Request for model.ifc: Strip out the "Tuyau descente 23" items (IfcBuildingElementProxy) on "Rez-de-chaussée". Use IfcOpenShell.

First a look at what the model holds.

```python
import ifcopenshell
import ifcopenshell.util.element

model = ifcopenshell.open("model.ifc")
print(model.schema)
storey = next(s for s in model.by_type("IfcBuildingStorey") if s.Name == "Rez-de-chaussée")
proxies = [e for e in ifcopenshell.util.element.get_decomposition(storey) if e.is_a("IfcBuildingElementProxy")]
seen = {}
for e in proxies:
    element_type = ifcopenshell.util.element.get_type(e)
    name = element_type.Name if element_type not in (None, e) else None
    seen[name] = seen.get(name, 0) + 1
for name, count in sorted(seen.items(), key=str):
    print(count, "x", name)
```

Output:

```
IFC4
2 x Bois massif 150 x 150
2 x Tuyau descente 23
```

```python
import ifcopenshell
import ifcopenshell.api.root
import ifcopenshell.util.element

model = ifcopenshell.open("model.ifc")

storey = next(s for s in model.by_type("IfcBuildingStorey") if s.Name == "Rez-de-chaussée")
proxies = [e for e in ifcopenshell.util.element.get_decomposition(storey) if e.is_a("IfcBuildingElementProxy")]
targets = [e for e in proxies if (t := ifcopenshell.util.element.get_type(e)) not in (None, e) and t.Name == "Tuyau descente 23"]

for e in targets:
    ifcopenshell.api.root.remove_product(model, product=e)
print(len(targets), "removed")

model.write("model_updated.ifc")
```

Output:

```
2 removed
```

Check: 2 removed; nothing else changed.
